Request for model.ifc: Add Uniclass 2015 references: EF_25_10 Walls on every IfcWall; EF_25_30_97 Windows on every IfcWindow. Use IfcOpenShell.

First a look at what the model holds.

```python
import ifcopenshell

model = ifcopenshell.open("model.ifc")
print(model.schema)
print("classifications:", [c.Name for c in model.by_type("IfcClassification")])
for ifc_class in ("IfcDoor", "IfcRoof", "IfcStair", "IfcWall", "IfcWindow"):
    print(ifc_class, len(model.by_type(ifc_class)))
```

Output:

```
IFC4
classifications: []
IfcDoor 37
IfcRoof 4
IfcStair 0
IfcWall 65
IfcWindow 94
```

```python
import ifcopenshell
import ifcopenshell.api.classification

model = ifcopenshell.open("model.ifc")

system = ifcopenshell.api.classification.add_classification(model, classification="Uniclass 2015")

codes = {
    "IfcWall": ("EF_25_10", "Walls"),
    "IfcWindow": ("EF_25_30_97", "Windows"),
}
for ifc_class, (code, name) in codes.items():
    products = model.by_type(ifc_class)
    ifcopenshell.api.classification.add_reference(
        model, products=products, classification=system, identification=code, name=name
    )
    print(code, len(products))

model.write("model-out.ifc")
```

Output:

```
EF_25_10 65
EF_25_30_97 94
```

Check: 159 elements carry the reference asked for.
